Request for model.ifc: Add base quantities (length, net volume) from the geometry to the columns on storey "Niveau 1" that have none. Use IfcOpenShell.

First a look at what the model holds.

```python
import ifcopenshell
import ifcopenshell.util.element
import ifcopenshell.util.unit

model = ifcopenshell.open("model.ifc")
print(model.schema)
for unit_type in ("LENGTHUNIT", "AREAUNIT", "VOLUMEUNIT"):
    print(unit_type, ifcopenshell.util.unit.calculate_unit_scale(model, unit_type))
storey = next(s for s in model.by_type("IfcBuildingStorey") if s.Name == "Niveau 1")
columns = [e for e in ifcopenshell.util.element.get_decomposition(storey) if e.is_a("IfcColumn")]
for e in sorted(columns, key=lambda e: e.id()):
    print(e.id(), e.is_a(), e.Name, list(ifcopenshell.util.element.get_psets(e, qtos_only=True)), sep=" | ")
```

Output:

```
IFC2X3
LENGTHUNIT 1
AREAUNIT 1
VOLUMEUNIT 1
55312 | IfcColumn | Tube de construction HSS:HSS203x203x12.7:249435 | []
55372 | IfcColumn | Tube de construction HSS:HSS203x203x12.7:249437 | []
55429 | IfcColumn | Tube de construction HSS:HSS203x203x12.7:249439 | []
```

```python
import ifcopenshell
import ifcopenshell.api.pset
import ifcopenshell.geom
import ifcopenshell.util.element
import ifcopenshell.util.shape
import ifcopenshell.util.unit

model = ifcopenshell.open("model.ifc")
unit_scale = ifcopenshell.util.unit.calculate_unit_scale(model)
volume_scale = ifcopenshell.util.unit.calculate_unit_scale(model, "VOLUMEUNIT")
settings = ifcopenshell.geom.settings()

storey = next(s for s in model.by_type("IfcBuildingStorey") if s.Name == "Niveau 1")
columns = [e for e in ifcopenshell.util.element.get_decomposition(storey) if e.is_a("IfcColumn")]

for e in sorted(columns, key=lambda e: e.id()):
    if ifcopenshell.util.element.get_psets(e, qtos_only=True, should_inherit=False):
        continue
    # Geometry comes back in metres, in the element's own axes.
    shape = ifcopenshell.geom.create_shape(settings, e)
    values = {
        "Length": ifcopenshell.util.shape.get_z(shape.geometry) / unit_scale,
        "NetVolume": ifcopenshell.util.shape.get_volume(shape.geometry) / volume_scale,
    }
    qto = ifcopenshell.api.pset.add_qto(model, product=e, name="BaseQuantities")
    ifcopenshell.api.pset.edit_qto(model, qto=qto, properties=values)
    print(e.id(), {k: round(v, 3) for k, v in values.items()})

model.write("model_updated.ifc")
```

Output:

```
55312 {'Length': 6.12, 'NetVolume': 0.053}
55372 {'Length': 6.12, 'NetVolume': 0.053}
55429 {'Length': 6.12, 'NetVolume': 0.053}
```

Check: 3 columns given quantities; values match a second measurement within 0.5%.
